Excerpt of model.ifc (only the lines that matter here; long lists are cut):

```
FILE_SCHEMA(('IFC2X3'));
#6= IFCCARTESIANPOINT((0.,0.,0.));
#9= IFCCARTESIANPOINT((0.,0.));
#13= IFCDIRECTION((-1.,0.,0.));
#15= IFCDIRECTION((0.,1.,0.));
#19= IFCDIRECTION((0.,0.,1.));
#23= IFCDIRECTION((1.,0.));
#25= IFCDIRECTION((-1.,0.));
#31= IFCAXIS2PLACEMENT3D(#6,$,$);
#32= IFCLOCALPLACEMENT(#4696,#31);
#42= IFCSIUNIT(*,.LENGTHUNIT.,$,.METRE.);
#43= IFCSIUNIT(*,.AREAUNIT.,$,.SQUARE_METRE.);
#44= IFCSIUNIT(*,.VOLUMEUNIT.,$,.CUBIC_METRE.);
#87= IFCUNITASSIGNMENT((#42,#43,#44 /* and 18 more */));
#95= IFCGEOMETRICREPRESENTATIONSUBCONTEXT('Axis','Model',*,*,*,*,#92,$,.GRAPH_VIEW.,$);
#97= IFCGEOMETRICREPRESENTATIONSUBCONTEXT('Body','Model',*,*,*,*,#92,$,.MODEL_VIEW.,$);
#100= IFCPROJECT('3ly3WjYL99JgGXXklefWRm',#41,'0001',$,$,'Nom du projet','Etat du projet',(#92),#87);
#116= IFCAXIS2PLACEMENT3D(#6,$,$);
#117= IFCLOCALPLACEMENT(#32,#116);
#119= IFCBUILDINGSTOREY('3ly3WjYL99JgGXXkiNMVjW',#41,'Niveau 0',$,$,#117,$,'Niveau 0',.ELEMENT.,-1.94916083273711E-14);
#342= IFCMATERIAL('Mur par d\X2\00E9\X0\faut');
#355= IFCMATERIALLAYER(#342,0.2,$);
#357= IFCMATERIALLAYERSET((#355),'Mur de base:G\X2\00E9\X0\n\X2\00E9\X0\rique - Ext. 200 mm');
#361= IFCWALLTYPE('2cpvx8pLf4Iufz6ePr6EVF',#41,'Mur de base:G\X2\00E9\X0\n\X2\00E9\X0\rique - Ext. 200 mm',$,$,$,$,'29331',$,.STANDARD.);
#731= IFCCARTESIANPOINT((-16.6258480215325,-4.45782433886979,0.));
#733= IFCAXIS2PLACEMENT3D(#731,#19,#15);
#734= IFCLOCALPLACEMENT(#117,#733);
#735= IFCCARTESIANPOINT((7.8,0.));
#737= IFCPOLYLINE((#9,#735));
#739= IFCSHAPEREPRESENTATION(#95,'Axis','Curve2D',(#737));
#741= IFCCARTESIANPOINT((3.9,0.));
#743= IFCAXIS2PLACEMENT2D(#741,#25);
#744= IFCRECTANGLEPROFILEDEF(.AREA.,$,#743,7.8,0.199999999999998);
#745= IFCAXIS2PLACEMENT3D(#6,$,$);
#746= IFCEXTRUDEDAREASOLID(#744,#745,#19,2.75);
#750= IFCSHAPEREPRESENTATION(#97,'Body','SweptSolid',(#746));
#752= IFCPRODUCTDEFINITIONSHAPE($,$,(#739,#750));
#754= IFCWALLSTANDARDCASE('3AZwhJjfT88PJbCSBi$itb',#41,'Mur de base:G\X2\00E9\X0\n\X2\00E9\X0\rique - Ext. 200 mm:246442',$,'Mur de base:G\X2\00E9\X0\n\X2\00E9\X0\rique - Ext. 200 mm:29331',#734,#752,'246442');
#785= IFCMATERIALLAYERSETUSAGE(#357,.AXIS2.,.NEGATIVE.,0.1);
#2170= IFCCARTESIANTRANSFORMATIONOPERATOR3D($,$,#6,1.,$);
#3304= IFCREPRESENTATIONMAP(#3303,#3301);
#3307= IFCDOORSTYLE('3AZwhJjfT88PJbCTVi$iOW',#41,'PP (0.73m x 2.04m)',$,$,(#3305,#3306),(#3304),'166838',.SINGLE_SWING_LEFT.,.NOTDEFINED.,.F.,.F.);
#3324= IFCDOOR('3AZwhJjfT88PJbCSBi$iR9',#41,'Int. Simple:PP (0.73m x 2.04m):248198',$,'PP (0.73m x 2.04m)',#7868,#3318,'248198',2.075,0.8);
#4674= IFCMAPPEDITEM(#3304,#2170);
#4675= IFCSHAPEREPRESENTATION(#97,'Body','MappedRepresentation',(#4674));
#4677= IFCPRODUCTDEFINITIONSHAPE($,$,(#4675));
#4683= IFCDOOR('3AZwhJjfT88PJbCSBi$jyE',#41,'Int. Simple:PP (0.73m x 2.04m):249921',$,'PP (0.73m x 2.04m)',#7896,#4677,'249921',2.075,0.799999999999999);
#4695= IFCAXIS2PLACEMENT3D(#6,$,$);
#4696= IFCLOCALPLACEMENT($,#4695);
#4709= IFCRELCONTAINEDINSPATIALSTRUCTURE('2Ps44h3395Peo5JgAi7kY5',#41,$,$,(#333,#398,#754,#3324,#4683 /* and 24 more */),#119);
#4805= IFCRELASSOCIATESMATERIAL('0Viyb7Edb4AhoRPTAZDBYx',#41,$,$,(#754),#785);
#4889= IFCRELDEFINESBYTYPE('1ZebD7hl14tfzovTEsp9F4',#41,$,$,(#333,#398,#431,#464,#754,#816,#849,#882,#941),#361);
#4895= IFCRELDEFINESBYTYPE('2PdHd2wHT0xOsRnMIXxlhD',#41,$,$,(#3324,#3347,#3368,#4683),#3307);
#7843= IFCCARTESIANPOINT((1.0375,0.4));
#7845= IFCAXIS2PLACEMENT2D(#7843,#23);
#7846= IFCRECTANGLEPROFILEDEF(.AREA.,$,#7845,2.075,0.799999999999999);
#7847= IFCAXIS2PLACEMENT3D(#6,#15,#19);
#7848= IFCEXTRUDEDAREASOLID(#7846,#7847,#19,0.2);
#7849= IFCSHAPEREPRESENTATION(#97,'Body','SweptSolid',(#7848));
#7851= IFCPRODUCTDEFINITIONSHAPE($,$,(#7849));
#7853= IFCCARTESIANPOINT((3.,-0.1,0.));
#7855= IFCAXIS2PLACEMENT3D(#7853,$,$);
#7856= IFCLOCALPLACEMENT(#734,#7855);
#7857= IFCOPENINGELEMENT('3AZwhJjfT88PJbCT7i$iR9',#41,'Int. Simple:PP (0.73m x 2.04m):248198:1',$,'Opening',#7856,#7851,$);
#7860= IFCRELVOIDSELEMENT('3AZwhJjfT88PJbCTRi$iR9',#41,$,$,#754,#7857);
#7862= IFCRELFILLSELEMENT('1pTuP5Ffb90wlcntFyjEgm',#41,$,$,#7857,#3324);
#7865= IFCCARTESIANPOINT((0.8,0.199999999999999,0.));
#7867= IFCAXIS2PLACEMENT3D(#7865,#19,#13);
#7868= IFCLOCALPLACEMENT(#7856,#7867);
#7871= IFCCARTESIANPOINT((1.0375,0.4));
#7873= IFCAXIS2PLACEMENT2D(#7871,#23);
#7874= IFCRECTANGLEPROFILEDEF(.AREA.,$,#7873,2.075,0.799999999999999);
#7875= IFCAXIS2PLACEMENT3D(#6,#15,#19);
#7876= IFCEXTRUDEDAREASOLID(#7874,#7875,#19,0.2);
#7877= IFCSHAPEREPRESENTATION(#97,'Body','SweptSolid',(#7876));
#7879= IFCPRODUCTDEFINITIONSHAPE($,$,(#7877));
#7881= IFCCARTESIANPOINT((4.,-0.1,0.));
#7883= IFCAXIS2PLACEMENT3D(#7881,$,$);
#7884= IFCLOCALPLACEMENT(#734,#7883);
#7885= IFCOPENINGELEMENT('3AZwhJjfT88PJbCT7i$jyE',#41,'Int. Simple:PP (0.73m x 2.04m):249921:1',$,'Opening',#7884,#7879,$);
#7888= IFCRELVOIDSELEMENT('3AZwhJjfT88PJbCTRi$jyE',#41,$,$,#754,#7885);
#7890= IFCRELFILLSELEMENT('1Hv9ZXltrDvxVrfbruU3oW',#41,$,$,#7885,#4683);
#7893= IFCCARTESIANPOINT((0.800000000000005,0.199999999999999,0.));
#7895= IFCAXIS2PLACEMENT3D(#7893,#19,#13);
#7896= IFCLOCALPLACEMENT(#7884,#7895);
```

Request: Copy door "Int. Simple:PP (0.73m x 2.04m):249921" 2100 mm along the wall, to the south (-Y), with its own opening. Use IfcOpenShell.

```python
import ifcopenshell
import ifcopenshell.api.feature
import ifcopenshell.api.geometry
import ifcopenshell.api.root
import ifcopenshell.geom
import ifcopenshell.util.element
import ifcopenshell.util.placement
import ifcopenshell.util.shape

model = ifcopenshell.open("model.ifc")
settings = ifcopenshell.geom.settings()


def volume(element):
    """Net volume in cubic metres, openings subtracted."""
    shape = ifcopenshell.geom.create_shape(settings, element)
    return ifcopenshell.util.shape.get_volume(shape.geometry)


def reuse_history(source, copy):
    """copy_class also copies each property set's owner history, people and application; keep the originals."""
    for rel in copy.IsDefinedBy:
        if rel.is_a("IfcRelDefinesByProperties") and (history := rel.RelatingPropertyDefinition.OwnerHistory):
            rel.RelatingPropertyDefinition.OwnerHistory = source.OwnerHistory
            ifcopenshell.util.element.remove_deep2(model, history)


door = model.by_id(4683)
opening = door.FillsVoids[0].RelatingOpeningElement
wall = opening.VoidsElements[0].RelatingBuildingElement
before = volume(wall)
shift = ifcopenshell.util.placement.get_local_placement(wall.ObjectPlacement)[:3, 0] * -2.1

# copy_class copies the void relationship, type, container and properties, but no geometry.
new_opening = ifcopenshell.api.root.copy_class(model, product=opening)
new_opening.Representation = ifcopenshell.util.element.copy_deep(
    model, opening.Representation, exclude=["IfcGeometricRepresentationContext", "IfcRepresentationMap"]
)
new_opening.Name = "Int. Simple:PP (0.73m x 2.04m)"
new_door = ifcopenshell.api.root.copy_class(model, product=door)
new_door.Representation = ifcopenshell.util.element.copy_deep(
    model, door.Representation, exclude=["IfcGeometricRepresentationContext", "IfcRepresentationMap"]
)
new_door.Name = "Int. Simple:PP (0.73m x 2.04m)"
new_door.Tag = None
reuse_history(door, new_door)
fills = ifcopenshell.api.feature.add_filling(model, opening=new_opening, element=new_door)
fills.OwnerHistory = new_door.OwnerHistory  # required in IFC2X3

for old, new in ((opening, new_opening), (door, new_door)):
    matrix = ifcopenshell.util.placement.get_local_placement(old.ObjectPlacement)
    matrix[:3, 3] += shift
    ifcopenshell.api.geometry.edit_object_placement(model, product=new, matrix=matrix, is_si=False)

after = volume(wall)

print(f"wall volume {before:.3f} -> {after:.3f} m3")

model.write("model-out.ifc")
```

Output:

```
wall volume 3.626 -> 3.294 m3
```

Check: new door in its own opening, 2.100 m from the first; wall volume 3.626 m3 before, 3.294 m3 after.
